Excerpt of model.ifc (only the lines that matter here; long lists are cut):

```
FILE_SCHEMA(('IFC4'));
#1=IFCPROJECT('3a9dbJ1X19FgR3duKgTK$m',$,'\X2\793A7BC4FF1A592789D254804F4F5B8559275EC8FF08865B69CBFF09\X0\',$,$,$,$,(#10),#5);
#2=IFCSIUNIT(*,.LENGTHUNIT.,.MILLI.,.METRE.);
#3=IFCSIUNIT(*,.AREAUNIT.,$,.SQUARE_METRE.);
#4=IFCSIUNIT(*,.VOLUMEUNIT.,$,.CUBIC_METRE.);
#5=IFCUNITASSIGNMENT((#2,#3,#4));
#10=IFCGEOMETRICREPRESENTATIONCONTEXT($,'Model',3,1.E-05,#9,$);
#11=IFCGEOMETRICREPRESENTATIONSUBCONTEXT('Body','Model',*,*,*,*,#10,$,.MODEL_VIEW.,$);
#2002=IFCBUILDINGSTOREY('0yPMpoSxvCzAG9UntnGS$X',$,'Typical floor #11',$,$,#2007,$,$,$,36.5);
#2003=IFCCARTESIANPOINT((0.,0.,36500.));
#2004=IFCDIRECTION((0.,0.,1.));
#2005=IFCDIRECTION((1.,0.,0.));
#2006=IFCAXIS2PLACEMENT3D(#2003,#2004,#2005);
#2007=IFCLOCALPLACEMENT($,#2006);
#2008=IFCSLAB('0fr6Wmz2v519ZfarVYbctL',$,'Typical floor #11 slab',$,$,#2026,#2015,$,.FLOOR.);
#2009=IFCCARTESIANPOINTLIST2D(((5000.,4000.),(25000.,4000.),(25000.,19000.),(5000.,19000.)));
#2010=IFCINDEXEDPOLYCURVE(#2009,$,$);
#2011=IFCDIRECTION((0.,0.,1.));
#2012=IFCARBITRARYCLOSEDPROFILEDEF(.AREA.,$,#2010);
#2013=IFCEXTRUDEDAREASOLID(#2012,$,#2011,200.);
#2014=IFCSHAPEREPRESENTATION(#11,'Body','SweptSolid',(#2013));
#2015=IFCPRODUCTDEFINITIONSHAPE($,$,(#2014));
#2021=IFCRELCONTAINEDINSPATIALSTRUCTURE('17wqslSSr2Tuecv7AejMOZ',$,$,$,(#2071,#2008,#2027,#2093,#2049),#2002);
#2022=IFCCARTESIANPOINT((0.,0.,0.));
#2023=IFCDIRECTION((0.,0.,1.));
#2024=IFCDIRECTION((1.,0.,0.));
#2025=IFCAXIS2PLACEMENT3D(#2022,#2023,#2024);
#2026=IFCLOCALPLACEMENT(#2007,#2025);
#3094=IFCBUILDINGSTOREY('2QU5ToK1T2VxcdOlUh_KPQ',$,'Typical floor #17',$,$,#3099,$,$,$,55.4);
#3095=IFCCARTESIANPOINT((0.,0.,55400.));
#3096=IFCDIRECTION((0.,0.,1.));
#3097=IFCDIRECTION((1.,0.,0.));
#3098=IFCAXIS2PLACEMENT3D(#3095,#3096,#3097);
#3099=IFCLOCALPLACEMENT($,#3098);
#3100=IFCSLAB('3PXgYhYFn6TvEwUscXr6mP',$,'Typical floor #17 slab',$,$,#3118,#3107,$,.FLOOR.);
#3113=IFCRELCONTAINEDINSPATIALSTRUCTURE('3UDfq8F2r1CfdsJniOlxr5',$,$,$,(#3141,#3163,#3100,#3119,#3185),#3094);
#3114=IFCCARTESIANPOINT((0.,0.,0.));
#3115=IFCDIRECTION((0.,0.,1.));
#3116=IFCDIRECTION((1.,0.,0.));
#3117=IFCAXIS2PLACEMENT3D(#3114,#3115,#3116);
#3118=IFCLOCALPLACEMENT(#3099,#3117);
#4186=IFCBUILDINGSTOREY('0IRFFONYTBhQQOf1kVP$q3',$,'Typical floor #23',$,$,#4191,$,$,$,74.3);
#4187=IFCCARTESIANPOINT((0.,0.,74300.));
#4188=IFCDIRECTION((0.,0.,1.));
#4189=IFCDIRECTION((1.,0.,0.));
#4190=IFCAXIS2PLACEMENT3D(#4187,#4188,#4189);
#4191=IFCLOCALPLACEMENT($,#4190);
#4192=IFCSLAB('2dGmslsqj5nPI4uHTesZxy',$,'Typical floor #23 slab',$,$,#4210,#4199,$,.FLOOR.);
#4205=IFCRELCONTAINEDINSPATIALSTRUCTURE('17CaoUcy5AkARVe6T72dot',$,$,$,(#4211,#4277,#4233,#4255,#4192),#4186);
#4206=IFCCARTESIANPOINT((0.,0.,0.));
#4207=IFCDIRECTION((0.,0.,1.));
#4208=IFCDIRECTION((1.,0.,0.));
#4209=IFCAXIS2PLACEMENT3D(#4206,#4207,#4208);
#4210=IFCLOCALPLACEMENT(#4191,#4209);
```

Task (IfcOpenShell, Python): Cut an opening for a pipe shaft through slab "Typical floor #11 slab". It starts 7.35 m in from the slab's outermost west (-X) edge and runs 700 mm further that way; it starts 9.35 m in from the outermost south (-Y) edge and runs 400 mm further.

```python
import numpy as np
import ifcopenshell
import ifcopenshell.api.feature
import ifcopenshell.api.geometry
import ifcopenshell.api.root
import ifcopenshell.geom
import ifcopenshell.util.placement
import ifcopenshell.util.representation
import ifcopenshell.util.shape
import ifcopenshell.util.unit

model = ifcopenshell.open("model.ifc")
unit_scale = ifcopenshell.util.unit.calculate_unit_scale(model)
settings = ifcopenshell.geom.settings()


def volume(element):
    """Net volume in cubic metres, openings subtracted."""
    shape = ifcopenshell.geom.create_shape(settings, element)
    return ifcopenshell.util.shape.get_volume(shape.geometry)


slab = model.by_guid("0fr6Wmz2v519ZfarVYbctL")
before = volume(slab)

# Extent in the slab's own axes, in metres. The edges named are its -X and -Y sides.
slab_shape = ifcopenshell.geom.create_shape(settings, slab)
vertices = ifcopenshell.util.shape.get_vertices(slab_shape.geometry)
x_min, y_min, bottom = vertices.min(axis=0)
top = vertices[:, 2].max()

opening = ifcopenshell.api.root.create_entity(model, ifc_class="IfcOpeningElement", name="Pipe shaft opening", predefined_type="OPENING")
context = ifcopenshell.util.representation.get_context(model, "Model", "Body", "MODEL_VIEW")
width, depth = 0.7, 0.4
outline = [(0.0, 0.0), (width, 0.0), (width, depth), (0.0, depth), (0.0, 0.0)]
# Overshoot both faces by 50 mm so the cut is clean.
shape = ifcopenshell.api.geometry.add_slab_representation(
    model, context=context, depth=top - bottom + 0.1, polyline=outline
)
ifcopenshell.api.geometry.assign_representation(model, product=opening, representation=shape)

matrix = ifcopenshell.util.placement.get_local_placement(slab.ObjectPlacement)
matrix[:, 3] = matrix @ np.append(np.array([x_min + 7.35, y_min + 9.35, bottom - 0.05]) / unit_scale, 1.0)
ifcopenshell.api.geometry.edit_object_placement(model, product=opening, matrix=matrix, is_si=False)
ifcopenshell.api.feature.add_feature(model, feature=opening, element=slab)

after = volume(slab)

print(f"slab volume {before:.3f} -> {after:.3f} m3")

model.write("model_v2.ifc")
```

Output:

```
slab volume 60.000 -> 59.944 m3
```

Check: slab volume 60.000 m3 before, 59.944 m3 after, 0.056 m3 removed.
